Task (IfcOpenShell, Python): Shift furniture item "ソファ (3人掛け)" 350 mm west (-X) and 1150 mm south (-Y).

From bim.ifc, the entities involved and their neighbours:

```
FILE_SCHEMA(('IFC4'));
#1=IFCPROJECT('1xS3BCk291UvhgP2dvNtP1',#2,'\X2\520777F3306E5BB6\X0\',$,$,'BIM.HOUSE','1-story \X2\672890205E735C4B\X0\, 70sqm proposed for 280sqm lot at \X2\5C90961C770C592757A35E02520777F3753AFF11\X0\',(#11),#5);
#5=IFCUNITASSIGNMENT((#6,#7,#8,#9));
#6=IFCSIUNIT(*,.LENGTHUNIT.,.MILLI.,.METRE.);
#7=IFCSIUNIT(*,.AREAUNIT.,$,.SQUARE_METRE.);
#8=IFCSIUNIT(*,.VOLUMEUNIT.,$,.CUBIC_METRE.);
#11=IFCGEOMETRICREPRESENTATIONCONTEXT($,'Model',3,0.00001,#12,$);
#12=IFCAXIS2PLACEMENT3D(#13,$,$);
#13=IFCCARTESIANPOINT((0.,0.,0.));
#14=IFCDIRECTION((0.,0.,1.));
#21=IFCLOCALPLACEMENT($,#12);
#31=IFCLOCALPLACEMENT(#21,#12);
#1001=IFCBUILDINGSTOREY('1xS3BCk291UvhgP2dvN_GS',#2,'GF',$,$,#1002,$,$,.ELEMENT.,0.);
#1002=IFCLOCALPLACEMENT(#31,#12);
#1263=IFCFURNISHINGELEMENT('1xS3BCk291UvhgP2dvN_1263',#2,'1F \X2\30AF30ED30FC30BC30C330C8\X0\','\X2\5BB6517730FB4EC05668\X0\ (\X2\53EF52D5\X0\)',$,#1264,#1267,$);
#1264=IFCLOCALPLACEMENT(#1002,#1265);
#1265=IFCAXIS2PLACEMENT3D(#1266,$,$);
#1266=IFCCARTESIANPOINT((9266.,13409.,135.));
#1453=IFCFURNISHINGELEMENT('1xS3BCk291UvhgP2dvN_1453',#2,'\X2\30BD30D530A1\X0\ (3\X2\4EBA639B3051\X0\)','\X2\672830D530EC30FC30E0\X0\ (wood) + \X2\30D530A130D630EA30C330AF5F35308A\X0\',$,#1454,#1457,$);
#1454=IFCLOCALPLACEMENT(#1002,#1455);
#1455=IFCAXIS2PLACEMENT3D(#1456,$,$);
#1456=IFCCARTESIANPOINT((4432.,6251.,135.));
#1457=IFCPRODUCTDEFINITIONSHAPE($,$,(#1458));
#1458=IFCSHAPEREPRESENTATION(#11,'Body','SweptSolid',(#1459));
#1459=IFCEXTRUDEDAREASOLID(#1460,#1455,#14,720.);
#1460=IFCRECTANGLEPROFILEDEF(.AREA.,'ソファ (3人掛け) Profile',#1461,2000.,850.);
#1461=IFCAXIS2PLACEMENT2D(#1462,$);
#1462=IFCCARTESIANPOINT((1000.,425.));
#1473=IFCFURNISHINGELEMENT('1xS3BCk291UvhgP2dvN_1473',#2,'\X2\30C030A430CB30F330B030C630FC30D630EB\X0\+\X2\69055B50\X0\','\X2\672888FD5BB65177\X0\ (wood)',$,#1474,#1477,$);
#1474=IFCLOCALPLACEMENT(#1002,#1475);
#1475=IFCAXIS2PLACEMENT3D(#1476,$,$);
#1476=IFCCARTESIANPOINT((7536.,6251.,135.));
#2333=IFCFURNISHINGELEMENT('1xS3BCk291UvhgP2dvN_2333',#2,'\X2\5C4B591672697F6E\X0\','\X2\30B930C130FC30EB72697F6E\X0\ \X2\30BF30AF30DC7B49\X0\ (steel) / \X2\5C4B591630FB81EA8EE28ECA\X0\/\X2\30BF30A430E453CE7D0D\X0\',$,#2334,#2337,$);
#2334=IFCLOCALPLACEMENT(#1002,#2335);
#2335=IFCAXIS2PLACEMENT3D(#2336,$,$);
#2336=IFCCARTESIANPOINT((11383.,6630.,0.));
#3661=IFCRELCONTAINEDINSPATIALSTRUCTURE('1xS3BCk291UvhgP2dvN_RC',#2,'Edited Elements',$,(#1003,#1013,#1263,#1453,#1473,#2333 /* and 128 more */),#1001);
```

```python
import ifcopenshell
import ifcopenshell.api.geometry
import ifcopenshell.util.placement
import ifcopenshell.util.unit

model = ifcopenshell.open("bim.ifc")
unit_scale = ifcopenshell.util.unit.calculate_unit_scale(model)

item = model.by_guid("1xS3BCk291UvhgP2dvN_1453")
matrix = ifcopenshell.util.placement.get_local_placement(item.ObjectPlacement)
matrix[0, 3] -= 0.35 / unit_scale
matrix[1, 3] -= 1.15 / unit_scale
ifcopenshell.api.geometry.edit_object_placement(model, product=item, matrix=matrix, is_si=False)

print(ifcopenshell.util.placement.get_local_placement(item.ObjectPlacement).round(3) + 0.0)

model.write("bim_edited.ifc")
```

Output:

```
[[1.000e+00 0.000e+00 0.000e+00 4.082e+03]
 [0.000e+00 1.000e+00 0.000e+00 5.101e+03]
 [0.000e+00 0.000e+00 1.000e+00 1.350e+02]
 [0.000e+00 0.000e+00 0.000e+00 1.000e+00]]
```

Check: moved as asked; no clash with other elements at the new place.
